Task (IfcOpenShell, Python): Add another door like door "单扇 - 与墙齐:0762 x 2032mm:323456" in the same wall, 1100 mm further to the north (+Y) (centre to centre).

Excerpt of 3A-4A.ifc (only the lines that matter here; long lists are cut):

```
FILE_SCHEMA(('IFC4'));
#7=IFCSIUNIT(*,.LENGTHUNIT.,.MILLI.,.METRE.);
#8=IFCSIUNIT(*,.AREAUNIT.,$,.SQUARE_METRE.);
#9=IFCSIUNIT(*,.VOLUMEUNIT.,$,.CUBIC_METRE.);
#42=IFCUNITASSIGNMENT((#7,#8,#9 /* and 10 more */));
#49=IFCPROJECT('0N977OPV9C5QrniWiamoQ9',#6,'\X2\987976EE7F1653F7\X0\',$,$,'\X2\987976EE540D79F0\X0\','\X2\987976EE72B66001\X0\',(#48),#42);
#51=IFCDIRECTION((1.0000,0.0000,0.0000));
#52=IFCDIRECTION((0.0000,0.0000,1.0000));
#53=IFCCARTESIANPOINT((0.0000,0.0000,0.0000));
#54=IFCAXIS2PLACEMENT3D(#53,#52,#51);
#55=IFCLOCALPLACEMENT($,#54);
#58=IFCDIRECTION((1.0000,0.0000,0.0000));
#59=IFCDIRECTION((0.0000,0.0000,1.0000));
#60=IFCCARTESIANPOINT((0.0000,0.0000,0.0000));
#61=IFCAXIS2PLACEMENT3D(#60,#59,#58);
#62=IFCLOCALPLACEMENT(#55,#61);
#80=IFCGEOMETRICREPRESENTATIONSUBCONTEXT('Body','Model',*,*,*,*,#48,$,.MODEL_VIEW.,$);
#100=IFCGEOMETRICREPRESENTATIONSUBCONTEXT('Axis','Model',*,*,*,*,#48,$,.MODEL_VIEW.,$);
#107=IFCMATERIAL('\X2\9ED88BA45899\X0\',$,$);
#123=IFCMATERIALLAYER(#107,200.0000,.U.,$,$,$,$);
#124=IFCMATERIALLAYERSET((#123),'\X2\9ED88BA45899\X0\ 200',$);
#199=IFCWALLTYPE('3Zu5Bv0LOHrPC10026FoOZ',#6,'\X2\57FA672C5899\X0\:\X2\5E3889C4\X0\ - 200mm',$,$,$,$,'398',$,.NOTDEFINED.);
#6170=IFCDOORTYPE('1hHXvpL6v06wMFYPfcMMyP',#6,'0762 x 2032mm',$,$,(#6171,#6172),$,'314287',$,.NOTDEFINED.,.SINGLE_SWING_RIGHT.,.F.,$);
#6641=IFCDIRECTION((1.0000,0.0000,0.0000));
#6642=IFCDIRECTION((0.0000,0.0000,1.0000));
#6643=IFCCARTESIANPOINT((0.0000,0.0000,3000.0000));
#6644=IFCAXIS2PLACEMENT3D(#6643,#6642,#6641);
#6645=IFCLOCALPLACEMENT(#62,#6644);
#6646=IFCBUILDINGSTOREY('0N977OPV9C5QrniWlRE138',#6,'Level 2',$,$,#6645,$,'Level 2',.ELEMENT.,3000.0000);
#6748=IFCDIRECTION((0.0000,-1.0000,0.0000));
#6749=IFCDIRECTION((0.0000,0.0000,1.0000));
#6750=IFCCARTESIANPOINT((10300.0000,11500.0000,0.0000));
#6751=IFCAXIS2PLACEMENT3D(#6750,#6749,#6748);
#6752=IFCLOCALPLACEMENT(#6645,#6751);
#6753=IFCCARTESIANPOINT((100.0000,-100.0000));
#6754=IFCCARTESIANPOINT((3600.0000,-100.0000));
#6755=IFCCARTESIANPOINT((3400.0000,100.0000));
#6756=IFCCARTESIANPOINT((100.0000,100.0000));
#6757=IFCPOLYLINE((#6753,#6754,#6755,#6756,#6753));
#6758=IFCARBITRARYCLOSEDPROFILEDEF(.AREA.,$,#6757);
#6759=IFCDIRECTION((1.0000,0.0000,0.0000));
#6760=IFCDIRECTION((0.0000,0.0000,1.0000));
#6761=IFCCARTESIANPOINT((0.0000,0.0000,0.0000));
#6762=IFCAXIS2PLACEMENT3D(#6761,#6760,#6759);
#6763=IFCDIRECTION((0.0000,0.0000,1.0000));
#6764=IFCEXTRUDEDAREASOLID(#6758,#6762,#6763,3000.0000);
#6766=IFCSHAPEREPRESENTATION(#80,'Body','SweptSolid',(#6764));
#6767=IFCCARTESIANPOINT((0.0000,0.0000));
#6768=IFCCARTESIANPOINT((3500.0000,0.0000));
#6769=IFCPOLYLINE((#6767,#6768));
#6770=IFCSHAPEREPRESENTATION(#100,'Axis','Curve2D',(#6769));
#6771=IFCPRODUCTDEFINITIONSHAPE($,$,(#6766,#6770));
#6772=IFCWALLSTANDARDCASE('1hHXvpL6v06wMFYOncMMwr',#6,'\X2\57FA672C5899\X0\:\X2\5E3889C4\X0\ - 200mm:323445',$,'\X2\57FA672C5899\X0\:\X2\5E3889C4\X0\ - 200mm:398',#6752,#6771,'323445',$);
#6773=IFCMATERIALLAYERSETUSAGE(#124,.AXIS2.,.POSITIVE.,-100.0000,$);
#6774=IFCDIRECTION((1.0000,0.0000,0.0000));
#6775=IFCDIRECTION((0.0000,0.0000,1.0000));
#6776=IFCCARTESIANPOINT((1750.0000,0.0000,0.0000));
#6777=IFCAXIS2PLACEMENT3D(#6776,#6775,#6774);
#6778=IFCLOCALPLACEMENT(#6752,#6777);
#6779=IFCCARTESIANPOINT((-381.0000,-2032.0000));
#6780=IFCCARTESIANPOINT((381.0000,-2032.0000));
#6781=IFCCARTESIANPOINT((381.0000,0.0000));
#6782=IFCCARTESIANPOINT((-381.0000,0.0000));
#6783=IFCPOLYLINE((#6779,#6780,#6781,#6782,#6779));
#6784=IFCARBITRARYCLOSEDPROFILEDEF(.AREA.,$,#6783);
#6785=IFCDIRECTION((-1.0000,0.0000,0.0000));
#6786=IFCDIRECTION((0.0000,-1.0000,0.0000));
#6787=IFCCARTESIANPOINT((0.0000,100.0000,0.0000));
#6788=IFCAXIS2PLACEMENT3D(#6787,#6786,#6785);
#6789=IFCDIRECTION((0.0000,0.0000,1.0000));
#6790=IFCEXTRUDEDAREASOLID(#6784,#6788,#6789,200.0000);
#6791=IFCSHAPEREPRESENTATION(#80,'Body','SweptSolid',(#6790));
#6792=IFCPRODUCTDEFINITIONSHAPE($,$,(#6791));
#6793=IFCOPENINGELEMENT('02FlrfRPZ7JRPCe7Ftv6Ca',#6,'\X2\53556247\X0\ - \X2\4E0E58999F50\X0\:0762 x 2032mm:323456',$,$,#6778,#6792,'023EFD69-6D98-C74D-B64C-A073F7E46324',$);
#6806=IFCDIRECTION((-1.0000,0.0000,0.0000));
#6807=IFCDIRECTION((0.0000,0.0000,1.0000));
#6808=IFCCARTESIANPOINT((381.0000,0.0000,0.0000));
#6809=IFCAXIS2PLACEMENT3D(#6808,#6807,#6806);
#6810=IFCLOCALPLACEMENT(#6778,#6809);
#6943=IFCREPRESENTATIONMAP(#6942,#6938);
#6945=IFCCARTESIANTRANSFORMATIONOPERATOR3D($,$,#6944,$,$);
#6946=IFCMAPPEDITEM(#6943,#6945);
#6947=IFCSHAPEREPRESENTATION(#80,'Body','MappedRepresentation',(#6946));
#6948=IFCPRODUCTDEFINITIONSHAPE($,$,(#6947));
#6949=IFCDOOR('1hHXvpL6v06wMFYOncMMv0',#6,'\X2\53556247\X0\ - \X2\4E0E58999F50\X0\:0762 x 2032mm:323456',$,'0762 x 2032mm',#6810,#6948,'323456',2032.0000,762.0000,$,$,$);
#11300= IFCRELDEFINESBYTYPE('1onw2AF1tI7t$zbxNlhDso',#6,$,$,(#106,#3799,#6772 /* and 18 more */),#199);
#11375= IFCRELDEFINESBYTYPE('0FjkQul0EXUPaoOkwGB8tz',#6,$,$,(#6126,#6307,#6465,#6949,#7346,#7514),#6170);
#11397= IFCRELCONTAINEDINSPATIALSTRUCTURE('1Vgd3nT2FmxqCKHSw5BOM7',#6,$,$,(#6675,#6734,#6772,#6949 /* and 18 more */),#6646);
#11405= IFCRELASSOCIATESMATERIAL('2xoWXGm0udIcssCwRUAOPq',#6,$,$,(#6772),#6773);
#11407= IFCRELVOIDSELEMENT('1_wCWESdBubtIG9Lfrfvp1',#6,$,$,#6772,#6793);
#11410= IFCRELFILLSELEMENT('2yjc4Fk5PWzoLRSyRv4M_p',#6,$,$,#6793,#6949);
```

```python
import ifcopenshell
import ifcopenshell.api.feature
import ifcopenshell.api.geometry
import ifcopenshell.api.root
import ifcopenshell.geom
import ifcopenshell.util.element
import ifcopenshell.util.placement
import ifcopenshell.util.shape
import ifcopenshell.util.unit

model = ifcopenshell.open("3A-4A.ifc")
unit_scale = ifcopenshell.util.unit.calculate_unit_scale(model)
settings = ifcopenshell.geom.settings()


def volume(element):
    """Net volume in cubic metres, openings subtracted."""
    shape = ifcopenshell.geom.create_shape(settings, element)
    return ifcopenshell.util.shape.get_volume(shape.geometry)


def reuse_history(source, copy):
    """copy_class also copies each property set's owner history, people and application; keep the originals."""
    for rel in copy.IsDefinedBy:
        if rel.is_a("IfcRelDefinesByProperties") and (history := rel.RelatingPropertyDefinition.OwnerHistory):
            rel.RelatingPropertyDefinition.OwnerHistory = source.OwnerHistory
            ifcopenshell.util.element.remove_deep2(model, history)


door = model.by_guid("1hHXvpL6v06wMFYOncMMv0")
opening = door.FillsVoids[0].RelatingOpeningElement
wall = opening.VoidsElements[0].RelatingBuildingElement
before = volume(wall)
shift = ifcopenshell.util.placement.get_local_placement(wall.ObjectPlacement)[:3, 0] * -1.1 / unit_scale

# copy_class copies the void relationship, type, container and properties, but no geometry.
new_opening = ifcopenshell.api.root.copy_class(model, product=opening)
new_opening.Representation = ifcopenshell.util.element.copy_deep(
    model, opening.Representation, exclude=["IfcGeometricRepresentationContext", "IfcRepresentationMap"]
)
new_opening.Name = "单扇 - 与墙齐:0762 x 2032mm"
new_opening.Tag = None
new_door = ifcopenshell.api.root.copy_class(model, product=door)
new_door.Representation = ifcopenshell.util.element.copy_deep(
    model, door.Representation, exclude=["IfcGeometricRepresentationContext", "IfcRepresentationMap"]
)
new_door.Name = "单扇 - 与墙齐:0762 x 2032mm"
new_door.Tag = None
reuse_history(door, new_door)
ifcopenshell.api.feature.add_filling(model, opening=new_opening, element=new_door)

for old, new in ((opening, new_opening), (door, new_door)):
    matrix = ifcopenshell.util.placement.get_local_placement(old.ObjectPlacement)
    matrix[:3, 3] += shift
    ifcopenshell.api.geometry.edit_object_placement(model, product=new, matrix=matrix, is_si=False)

after = volume(wall)

print(f"wall volume {before:.3f} -> {after:.3f} m3")

model.write("3A-4A_edited.ifc")
```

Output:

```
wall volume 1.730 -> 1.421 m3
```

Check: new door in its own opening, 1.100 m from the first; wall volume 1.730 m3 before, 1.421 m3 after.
